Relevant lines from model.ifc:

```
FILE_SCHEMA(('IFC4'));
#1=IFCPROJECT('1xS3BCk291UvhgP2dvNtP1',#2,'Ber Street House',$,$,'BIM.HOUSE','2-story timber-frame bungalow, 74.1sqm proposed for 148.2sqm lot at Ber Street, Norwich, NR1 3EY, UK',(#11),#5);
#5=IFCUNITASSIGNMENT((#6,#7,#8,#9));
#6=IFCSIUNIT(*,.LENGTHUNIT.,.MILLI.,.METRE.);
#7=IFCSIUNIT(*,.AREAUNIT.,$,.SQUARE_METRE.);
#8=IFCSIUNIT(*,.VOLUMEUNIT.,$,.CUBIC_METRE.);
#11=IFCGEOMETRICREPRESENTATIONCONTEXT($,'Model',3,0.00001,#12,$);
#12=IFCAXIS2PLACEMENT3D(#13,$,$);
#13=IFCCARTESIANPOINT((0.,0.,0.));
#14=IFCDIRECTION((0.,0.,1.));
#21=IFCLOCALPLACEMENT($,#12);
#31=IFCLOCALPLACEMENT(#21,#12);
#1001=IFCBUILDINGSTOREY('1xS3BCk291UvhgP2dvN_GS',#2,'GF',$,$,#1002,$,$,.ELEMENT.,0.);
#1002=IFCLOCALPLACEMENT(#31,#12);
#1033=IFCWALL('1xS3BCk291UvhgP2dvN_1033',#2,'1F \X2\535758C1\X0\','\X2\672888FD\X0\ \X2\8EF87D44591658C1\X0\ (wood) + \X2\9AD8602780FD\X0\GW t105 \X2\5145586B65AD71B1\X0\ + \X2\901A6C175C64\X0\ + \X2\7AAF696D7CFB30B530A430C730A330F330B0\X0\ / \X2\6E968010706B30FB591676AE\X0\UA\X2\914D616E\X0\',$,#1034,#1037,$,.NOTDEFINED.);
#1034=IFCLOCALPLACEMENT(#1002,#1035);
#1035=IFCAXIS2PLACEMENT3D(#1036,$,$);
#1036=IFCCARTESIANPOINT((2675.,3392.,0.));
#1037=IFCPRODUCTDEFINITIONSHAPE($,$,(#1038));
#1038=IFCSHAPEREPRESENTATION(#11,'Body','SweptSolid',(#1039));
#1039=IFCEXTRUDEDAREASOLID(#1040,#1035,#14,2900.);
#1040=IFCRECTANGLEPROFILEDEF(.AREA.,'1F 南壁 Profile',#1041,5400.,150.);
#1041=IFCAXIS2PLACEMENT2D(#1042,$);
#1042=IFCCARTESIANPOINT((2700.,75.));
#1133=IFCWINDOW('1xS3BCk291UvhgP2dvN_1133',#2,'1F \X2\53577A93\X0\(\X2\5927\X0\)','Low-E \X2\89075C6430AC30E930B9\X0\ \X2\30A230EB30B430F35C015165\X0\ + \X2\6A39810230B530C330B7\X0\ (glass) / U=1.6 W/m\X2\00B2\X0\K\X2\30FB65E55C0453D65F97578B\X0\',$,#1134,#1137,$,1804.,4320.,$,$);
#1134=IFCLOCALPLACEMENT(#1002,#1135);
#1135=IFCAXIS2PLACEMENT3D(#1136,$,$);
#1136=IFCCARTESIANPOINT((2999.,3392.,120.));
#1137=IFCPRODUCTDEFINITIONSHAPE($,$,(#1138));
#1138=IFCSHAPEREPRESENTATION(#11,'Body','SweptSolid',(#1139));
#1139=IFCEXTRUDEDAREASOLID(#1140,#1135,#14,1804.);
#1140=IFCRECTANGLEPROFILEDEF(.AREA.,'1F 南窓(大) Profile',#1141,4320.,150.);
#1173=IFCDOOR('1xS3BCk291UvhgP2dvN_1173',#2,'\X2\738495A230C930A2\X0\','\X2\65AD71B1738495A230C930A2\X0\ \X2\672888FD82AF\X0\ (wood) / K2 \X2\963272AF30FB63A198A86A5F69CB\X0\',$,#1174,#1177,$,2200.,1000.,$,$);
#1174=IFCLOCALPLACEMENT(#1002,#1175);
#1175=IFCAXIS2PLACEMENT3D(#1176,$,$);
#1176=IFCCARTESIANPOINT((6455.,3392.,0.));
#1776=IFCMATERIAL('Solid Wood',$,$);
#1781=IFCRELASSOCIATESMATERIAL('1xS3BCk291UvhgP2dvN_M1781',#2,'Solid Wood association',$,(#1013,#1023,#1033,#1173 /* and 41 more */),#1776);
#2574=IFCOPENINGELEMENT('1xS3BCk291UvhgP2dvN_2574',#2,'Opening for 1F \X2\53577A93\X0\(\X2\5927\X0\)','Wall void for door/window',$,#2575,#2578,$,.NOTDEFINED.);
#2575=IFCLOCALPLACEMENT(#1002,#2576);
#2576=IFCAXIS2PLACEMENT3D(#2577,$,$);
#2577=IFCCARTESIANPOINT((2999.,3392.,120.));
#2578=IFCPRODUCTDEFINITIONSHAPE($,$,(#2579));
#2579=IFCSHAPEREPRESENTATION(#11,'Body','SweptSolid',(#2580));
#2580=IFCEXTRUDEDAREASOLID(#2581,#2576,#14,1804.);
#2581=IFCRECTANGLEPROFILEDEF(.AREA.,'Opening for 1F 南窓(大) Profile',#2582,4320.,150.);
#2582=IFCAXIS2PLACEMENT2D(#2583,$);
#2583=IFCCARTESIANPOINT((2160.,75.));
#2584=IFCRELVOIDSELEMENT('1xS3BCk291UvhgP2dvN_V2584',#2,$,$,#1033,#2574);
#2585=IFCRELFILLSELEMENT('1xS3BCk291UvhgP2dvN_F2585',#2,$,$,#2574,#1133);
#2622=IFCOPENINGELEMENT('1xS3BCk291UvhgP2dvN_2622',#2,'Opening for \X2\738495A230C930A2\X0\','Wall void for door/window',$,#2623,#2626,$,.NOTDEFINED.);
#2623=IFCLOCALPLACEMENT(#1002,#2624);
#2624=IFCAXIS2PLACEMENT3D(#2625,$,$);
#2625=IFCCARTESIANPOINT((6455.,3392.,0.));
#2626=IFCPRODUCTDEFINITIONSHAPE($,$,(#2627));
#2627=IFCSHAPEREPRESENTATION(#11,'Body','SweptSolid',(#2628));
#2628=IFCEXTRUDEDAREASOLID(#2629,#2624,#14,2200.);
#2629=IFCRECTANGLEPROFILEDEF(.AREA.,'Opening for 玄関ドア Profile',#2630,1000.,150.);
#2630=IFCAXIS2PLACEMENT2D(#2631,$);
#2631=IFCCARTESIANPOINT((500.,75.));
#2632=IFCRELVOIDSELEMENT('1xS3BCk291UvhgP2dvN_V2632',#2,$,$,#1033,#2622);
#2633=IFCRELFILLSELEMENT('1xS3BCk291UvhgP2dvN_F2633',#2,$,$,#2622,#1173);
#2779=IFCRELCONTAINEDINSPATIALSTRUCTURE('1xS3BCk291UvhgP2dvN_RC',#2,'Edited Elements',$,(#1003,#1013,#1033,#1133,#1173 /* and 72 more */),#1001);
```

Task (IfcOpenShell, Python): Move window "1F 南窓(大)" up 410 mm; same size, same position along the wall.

```python
import numpy as np
import ifcopenshell
import ifcopenshell.api.geometry
import ifcopenshell.util.placement
import ifcopenshell.util.unit

model = ifcopenshell.open("model.ifc")
unit_scale = ifcopenshell.util.unit.calculate_unit_scale(model)

window = model.by_guid("1xS3BCk291UvhgP2dvN_1133")
opening = window.FillsVoids[0].RelatingOpeningElement
dz = 0.41 / unit_scale

shift = np.array([0.0, 0.0, dz])
# The window is not placed relative to its opening, so move both.
for product in (opening, window):
    matrix = ifcopenshell.util.placement.get_local_placement(product.ObjectPlacement)
    matrix[:3, 3] += shift
    ifcopenshell.api.geometry.edit_object_placement(model, product=product, matrix=matrix, is_si=False)

print(f"moved by {dz * unit_scale:+.3f} m")

model.write("model_updated.ifc")
```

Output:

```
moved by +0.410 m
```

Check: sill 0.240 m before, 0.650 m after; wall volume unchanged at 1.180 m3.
